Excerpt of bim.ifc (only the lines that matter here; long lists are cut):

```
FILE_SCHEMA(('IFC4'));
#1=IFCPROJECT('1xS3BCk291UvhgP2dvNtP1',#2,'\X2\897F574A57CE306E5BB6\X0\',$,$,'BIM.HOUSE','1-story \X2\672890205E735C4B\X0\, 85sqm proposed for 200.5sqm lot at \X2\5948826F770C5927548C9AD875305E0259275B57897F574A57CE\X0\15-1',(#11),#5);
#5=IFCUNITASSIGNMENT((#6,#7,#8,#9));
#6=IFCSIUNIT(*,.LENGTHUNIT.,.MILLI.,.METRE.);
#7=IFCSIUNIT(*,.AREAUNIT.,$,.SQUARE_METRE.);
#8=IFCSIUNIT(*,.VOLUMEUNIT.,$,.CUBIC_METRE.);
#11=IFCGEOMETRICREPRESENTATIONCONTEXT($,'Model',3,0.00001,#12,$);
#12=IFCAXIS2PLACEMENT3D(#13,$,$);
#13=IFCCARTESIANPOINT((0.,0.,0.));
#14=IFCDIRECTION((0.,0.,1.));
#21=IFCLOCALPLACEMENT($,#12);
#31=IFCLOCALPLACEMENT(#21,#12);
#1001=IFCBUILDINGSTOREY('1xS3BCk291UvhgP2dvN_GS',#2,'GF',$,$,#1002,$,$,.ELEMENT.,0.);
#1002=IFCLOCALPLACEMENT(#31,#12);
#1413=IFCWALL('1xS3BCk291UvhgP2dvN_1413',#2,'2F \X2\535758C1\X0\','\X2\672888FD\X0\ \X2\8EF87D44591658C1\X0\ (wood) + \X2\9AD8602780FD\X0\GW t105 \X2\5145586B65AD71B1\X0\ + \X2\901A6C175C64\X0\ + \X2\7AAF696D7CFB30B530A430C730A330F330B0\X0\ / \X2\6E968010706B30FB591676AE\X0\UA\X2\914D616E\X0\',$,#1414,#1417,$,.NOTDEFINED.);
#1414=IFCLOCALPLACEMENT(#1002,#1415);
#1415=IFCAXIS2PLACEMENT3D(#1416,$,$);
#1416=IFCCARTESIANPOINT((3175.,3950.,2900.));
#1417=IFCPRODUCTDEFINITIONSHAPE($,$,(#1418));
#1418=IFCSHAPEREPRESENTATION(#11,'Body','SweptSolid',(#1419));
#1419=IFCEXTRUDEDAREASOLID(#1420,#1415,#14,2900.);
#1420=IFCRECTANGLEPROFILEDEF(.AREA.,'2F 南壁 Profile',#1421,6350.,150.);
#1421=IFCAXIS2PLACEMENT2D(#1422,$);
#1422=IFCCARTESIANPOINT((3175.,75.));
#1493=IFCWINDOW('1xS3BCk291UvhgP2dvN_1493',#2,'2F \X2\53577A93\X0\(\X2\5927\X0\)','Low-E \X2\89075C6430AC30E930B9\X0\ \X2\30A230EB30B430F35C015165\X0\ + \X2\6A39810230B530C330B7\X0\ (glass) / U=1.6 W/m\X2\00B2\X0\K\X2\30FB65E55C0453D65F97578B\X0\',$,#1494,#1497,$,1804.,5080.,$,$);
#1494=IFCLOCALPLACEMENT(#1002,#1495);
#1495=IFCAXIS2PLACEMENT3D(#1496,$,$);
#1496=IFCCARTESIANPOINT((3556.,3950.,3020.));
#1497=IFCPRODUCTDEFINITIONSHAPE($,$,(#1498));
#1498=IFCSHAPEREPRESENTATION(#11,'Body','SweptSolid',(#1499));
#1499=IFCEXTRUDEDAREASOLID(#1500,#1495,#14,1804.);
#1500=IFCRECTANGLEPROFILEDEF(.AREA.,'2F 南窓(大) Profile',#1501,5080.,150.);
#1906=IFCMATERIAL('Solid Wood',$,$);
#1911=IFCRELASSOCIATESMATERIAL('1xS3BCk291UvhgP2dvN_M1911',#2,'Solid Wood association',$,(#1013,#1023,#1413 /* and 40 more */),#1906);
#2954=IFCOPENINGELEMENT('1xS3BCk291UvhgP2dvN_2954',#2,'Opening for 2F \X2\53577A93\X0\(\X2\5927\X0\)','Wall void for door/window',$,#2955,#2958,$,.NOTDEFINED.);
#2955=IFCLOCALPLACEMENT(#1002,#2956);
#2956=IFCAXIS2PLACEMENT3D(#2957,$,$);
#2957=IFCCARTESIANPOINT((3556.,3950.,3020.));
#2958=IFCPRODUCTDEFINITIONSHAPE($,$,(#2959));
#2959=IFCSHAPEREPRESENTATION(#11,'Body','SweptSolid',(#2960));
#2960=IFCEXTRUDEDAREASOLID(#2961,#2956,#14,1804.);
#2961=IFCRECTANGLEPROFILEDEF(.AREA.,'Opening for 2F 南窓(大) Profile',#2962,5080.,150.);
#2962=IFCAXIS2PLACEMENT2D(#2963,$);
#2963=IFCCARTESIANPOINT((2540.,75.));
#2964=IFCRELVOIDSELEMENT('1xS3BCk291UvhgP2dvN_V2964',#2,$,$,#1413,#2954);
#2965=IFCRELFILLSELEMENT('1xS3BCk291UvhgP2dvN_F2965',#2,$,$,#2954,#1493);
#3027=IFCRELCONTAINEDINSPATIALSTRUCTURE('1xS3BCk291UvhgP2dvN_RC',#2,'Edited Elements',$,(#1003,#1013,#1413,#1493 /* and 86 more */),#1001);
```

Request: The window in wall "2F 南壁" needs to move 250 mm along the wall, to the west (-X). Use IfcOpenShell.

```python
import ifcopenshell
import ifcopenshell.api.geometry
import ifcopenshell.util.placement
import ifcopenshell.util.unit

model = ifcopenshell.open("bim.ifc")
unit_scale = ifcopenshell.util.unit.calculate_unit_scale(model)

window = model.by_guid("1xS3BCk291UvhgP2dvN_1493")
opening = window.FillsVoids[0].RelatingOpeningElement
wall = opening.VoidsElements[0].RelatingBuildingElement

wall_matrix = ifcopenshell.util.placement.get_local_placement(wall.ObjectPlacement)
shift = wall_matrix[:3, 0] * -0.25 / unit_scale
before = ifcopenshell.util.placement.get_local_placement(window.ObjectPlacement)[:3, 3].copy()

# The window is not placed relative to its opening, so move both.
for product in (opening, window):
    matrix = ifcopenshell.util.placement.get_local_placement(product.ObjectPlacement)
    matrix[:3, 3] += shift
    ifcopenshell.api.geometry.edit_object_placement(model, product=product, matrix=matrix, is_si=False)

after = ifcopenshell.util.placement.get_local_placement(window.ObjectPlacement)[:3, 3]
print("window moved by", (after - before).round(3) + 0.0)

model.write("bim-out.ifc")
```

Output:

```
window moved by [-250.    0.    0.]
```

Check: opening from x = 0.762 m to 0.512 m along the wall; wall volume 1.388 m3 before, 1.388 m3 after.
